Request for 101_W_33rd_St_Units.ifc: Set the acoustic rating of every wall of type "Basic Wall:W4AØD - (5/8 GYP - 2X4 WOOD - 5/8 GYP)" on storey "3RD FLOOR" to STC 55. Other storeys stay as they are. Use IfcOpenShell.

First a look at what the model holds.

```python
import ifcopenshell
import ifcopenshell.util.element

model = ifcopenshell.open("101_W_33rd_St_Units.ifc")
print(model.schema)
storey = next(s for s in model.by_type("IfcBuildingStorey") if s.Name == "3RD FLOOR")
walls = [e for e in ifcopenshell.util.element.get_decomposition(storey) if e.is_a("IfcWall")]
seen = {}
for e in walls:
    element_type = ifcopenshell.util.element.get_type(e)
    key = (element_type.Name if element_type != e and element_type else None, ifcopenshell.util.element.get_pset(e, "Pset_WallCommon", "AcousticRating"))
    seen[key] = seen.get(key, 0) + 1
for (name, value), count in sorted(seen.items(), key=str):
    print(count, "x", name, "|", value)
```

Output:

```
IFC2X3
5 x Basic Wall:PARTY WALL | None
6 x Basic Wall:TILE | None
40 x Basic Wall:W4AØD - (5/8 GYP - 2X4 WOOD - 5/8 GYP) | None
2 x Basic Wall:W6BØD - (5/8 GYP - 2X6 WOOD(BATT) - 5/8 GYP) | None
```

```python
import ifcopenshell
import ifcopenshell.api.pset
import ifcopenshell.util.element

model = ifcopenshell.open("101_W_33rd_St_Units.ifc")

storey = next(s for s in model.by_type("IfcBuildingStorey") if s.Name == "3RD FLOOR")
walls = [e for e in ifcopenshell.util.element.get_decomposition(storey) if e.is_a("IfcWall")]

count = 0
for e in walls:
    element_type = ifcopenshell.util.element.get_type(e)
    if element_type in (None, e) or element_type.Name != "Basic Wall:W4AØD - (5/8 GYP - 2X4 WOOD - 5/8 GYP)":
        continue
    # add_pset returns the element's existing set when there is one.
    pset = ifcopenshell.api.pset.add_pset(model, product=e, name="Pset_WallCommon")
    ifcopenshell.api.pset.edit_pset(model, pset=pset, properties={"AcousticRating": "STC 55"})
    count += 1

print(count, "walls updated")

model.write("101_W_33rd_St_Units_edited.ifc")
```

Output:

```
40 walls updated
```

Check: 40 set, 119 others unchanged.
